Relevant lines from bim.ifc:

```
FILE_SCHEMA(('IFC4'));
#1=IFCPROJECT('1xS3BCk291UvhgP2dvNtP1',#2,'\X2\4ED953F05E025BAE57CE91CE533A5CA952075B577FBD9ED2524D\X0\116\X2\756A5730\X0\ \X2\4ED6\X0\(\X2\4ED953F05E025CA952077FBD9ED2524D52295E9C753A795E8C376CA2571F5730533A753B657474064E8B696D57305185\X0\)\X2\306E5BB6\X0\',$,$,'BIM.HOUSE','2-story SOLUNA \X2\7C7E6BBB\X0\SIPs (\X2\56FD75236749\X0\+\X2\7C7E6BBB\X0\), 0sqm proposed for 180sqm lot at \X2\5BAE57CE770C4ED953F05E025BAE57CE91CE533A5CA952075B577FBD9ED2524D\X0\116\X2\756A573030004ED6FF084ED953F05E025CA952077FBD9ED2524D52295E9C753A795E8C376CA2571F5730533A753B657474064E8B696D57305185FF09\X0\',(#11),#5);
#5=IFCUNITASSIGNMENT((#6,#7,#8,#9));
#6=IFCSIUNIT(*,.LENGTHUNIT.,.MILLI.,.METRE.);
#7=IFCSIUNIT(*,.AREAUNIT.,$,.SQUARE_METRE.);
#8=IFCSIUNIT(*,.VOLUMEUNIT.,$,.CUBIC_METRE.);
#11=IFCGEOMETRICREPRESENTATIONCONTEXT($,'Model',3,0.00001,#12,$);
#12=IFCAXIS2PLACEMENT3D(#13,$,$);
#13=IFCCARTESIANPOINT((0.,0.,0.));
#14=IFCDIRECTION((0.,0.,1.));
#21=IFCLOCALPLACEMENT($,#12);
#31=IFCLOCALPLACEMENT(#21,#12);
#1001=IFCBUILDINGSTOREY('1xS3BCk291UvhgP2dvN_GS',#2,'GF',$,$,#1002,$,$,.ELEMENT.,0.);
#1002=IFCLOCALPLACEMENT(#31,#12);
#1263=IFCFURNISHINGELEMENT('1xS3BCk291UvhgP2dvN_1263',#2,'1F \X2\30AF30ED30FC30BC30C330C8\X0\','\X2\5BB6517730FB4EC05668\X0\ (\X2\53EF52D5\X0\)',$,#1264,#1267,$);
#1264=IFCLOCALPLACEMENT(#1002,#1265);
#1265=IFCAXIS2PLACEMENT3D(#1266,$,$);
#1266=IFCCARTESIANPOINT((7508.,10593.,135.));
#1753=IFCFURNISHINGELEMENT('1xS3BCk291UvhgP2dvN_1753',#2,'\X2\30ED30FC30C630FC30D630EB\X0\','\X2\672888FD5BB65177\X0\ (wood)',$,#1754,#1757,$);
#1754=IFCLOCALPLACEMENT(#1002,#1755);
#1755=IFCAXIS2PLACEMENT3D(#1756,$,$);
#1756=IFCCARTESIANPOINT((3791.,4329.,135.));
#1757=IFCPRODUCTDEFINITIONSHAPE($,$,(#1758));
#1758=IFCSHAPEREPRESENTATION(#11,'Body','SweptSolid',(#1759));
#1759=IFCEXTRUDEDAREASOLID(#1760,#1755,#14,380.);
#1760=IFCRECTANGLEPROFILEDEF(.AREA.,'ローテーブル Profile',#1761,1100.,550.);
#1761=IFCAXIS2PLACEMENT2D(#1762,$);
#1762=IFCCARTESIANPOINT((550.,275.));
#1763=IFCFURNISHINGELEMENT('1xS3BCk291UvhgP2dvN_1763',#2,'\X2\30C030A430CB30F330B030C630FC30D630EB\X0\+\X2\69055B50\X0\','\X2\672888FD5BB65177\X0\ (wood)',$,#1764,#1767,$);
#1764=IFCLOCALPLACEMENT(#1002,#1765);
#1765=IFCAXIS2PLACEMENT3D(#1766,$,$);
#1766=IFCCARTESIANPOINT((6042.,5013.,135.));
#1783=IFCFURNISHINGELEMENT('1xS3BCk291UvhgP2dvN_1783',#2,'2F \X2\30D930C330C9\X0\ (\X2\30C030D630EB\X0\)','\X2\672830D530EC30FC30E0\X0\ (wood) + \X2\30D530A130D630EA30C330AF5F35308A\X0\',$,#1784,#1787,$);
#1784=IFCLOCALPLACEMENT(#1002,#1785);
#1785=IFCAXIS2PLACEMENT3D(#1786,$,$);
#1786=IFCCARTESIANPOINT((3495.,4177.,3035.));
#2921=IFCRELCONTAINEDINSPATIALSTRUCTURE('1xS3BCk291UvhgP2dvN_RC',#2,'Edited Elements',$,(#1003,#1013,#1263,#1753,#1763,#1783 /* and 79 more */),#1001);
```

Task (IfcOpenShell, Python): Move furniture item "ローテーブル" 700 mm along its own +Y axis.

```python
import ifcopenshell
import ifcopenshell.api.geometry
import ifcopenshell.util.placement

model = ifcopenshell.open("bim.ifc")

item = model.by_guid("1xS3BCk291UvhgP2dvN_1753")
matrix = ifcopenshell.util.placement.get_local_placement(item.ObjectPlacement)
matrix[:3, 3] += matrix[:3, 1] * 700.0
ifcopenshell.api.geometry.edit_object_placement(model, product=item, matrix=matrix, is_si=False)

print(ifcopenshell.util.placement.get_local_placement(item.ObjectPlacement).round(3) + 0.0)

model.write("bim_v2.ifc")
```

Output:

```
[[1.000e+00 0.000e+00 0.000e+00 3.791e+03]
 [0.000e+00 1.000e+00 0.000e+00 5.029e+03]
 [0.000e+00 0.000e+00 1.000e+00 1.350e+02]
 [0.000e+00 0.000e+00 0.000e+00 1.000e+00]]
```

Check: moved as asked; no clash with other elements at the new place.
